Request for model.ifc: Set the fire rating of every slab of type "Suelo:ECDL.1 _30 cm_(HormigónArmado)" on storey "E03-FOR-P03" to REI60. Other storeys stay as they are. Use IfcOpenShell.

First a look at what the model holds.

```python
import ifcopenshell
import ifcopenshell.util.element

model = ifcopenshell.open("model.ifc")
print(model.schema)
storey = next(s for s in model.by_type("IfcBuildingStorey") if s.Name == "E03-FOR-P03")
slabs = [e for e in ifcopenshell.util.element.get_decomposition(storey) if e.is_a("IfcSlab")]
seen = {}
for e in slabs:
    element_type = ifcopenshell.util.element.get_type(e)
    key = (element_type.Name if element_type != e and element_type else None, ifcopenshell.util.element.get_pset(e, "Pset_SlabCommon", "FireRating"))
    seen[key] = seen.get(key, 0) + 1
for (name, value), count in sorted(seen.items(), key=str):
    print(count, "x", name, "|", value)
```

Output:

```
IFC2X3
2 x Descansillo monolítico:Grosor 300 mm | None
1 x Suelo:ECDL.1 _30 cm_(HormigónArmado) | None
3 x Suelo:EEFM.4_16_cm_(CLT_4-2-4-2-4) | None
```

```python
import ifcopenshell
import ifcopenshell.api.pset
import ifcopenshell.util.element

model = ifcopenshell.open("model.ifc")

storey = next(s for s in model.by_type("IfcBuildingStorey") if s.Name == "E03-FOR-P03")
slabs = [e for e in ifcopenshell.util.element.get_decomposition(storey) if e.is_a("IfcSlab")]

count = 0
for e in slabs:
    element_type = ifcopenshell.util.element.get_type(e)
    if element_type in (None, e) or element_type.Name != "Suelo:ECDL.1 _30 cm_(HormigónArmado)":
        continue
    # add_pset returns the element's existing set when there is one.
    pset = ifcopenshell.api.pset.add_pset(model, product=e, name="Pset_SlabCommon")
    ifcopenshell.api.pset.edit_pset(model, pset=pset, properties={"FireRating": "REI60"})
    count += 1

print(count, "slabs updated")

model.write("model_updated.ifc")
```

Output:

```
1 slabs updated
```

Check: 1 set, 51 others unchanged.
